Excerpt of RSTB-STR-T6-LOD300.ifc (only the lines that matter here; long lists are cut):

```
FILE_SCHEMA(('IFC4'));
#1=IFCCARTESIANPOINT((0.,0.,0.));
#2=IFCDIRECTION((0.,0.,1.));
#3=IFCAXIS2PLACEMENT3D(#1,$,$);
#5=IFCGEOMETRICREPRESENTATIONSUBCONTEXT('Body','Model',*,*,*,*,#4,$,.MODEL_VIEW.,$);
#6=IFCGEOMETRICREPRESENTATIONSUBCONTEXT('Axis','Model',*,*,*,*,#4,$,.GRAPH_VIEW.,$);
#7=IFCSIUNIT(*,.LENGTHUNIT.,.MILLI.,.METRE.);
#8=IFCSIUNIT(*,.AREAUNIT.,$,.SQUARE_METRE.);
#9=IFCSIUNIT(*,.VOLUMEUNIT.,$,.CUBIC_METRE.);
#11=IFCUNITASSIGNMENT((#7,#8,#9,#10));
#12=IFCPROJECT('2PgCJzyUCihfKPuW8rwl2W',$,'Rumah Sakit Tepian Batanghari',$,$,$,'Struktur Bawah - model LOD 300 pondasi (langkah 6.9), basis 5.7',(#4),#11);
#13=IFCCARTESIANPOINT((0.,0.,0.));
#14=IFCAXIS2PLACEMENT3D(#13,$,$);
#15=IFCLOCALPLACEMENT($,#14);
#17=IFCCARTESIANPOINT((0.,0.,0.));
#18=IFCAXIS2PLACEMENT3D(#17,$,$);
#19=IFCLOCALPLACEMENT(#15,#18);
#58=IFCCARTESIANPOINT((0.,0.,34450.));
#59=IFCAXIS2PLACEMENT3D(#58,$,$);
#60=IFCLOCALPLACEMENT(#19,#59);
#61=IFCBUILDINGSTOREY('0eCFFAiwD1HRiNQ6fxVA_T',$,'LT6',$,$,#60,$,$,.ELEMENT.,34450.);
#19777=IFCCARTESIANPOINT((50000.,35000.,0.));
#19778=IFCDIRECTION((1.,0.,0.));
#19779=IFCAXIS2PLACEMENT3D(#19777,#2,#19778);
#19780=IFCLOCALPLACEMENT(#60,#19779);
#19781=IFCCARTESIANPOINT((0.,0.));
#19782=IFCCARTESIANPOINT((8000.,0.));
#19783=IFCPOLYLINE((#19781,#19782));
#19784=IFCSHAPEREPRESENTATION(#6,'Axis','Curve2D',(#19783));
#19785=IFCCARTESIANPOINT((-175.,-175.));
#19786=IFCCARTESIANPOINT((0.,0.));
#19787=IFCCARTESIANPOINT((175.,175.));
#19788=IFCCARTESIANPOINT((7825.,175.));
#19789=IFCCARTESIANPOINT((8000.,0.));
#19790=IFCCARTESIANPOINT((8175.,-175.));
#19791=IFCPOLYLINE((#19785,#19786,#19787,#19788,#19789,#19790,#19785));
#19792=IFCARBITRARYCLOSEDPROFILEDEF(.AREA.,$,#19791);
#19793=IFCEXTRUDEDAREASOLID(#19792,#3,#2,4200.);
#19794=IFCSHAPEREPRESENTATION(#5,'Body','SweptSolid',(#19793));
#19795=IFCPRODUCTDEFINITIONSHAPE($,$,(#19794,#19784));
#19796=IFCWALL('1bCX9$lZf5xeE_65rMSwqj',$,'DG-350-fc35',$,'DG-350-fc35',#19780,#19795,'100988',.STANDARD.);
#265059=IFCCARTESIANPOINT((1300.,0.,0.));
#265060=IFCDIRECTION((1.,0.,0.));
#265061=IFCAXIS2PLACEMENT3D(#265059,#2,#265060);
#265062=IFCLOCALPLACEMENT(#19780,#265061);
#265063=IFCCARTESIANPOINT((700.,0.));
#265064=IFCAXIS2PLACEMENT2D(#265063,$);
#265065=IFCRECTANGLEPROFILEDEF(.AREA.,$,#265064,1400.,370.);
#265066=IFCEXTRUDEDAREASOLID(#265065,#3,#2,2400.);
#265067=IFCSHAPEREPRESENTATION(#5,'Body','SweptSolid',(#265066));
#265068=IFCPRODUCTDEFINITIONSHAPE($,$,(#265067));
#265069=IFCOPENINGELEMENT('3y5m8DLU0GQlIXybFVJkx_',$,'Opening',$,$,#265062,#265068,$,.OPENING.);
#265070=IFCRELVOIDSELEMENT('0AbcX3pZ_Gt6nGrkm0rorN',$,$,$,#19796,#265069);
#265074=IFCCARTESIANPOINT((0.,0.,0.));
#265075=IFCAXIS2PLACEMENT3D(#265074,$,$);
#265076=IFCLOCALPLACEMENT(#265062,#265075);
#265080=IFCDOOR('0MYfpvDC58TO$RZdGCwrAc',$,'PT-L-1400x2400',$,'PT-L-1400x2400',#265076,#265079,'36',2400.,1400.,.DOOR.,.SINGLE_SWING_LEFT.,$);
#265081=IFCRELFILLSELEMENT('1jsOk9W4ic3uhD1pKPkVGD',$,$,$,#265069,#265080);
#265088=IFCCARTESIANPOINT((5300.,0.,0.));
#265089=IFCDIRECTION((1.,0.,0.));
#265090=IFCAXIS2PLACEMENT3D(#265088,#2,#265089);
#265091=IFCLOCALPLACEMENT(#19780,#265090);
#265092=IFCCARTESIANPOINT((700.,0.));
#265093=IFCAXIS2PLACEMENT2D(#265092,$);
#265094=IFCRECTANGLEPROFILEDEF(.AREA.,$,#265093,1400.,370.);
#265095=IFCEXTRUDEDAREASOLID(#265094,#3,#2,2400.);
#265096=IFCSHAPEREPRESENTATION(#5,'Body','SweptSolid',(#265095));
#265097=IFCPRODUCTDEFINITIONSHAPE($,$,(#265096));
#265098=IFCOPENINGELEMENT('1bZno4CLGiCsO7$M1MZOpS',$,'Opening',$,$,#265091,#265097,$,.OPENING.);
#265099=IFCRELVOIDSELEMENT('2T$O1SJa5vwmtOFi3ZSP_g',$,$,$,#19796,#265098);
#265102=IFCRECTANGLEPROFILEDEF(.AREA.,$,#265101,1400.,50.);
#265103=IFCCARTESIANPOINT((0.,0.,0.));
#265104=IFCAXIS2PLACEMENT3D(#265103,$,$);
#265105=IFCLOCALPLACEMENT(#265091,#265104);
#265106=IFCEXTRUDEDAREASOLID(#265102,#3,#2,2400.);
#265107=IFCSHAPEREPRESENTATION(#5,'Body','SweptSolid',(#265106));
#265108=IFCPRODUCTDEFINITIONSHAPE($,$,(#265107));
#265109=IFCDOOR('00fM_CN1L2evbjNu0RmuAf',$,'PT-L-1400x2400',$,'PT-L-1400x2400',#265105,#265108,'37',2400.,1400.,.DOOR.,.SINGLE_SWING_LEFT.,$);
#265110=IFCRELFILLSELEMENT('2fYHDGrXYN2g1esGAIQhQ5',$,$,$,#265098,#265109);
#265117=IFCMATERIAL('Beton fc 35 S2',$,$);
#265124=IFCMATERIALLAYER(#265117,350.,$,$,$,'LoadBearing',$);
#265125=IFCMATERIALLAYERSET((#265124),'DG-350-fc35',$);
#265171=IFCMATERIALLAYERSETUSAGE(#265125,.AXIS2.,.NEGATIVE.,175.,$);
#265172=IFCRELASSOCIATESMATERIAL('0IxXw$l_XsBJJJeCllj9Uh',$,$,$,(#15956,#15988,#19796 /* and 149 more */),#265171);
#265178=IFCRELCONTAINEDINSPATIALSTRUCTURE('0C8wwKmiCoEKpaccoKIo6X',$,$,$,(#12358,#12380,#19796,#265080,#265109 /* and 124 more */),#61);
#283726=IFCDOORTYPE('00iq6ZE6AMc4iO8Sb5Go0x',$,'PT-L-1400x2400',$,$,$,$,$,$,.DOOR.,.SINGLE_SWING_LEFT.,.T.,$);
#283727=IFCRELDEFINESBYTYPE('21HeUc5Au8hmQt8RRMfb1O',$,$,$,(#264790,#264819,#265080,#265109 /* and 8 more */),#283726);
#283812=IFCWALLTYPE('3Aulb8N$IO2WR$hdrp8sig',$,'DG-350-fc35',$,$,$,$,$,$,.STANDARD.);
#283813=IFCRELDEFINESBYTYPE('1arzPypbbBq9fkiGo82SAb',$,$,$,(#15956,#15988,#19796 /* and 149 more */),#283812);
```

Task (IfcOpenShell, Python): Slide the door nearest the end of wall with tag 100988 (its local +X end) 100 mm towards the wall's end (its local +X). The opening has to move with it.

```python
import ifcopenshell
import ifcopenshell.api.geometry
import ifcopenshell.util.placement
import ifcopenshell.util.unit

model = ifcopenshell.open("RSTB-STR-T6-LOD300.ifc")
unit_scale = ifcopenshell.util.unit.calculate_unit_scale(model)

door = model.by_guid("00fM_CN1L2evbjNu0RmuAf")
opening = door.FillsVoids[0].RelatingOpeningElement
wall = opening.VoidsElements[0].RelatingBuildingElement

wall_matrix = ifcopenshell.util.placement.get_local_placement(wall.ObjectPlacement)
shift = wall_matrix[:3, 0] * 0.1 / unit_scale
before = ifcopenshell.util.placement.get_local_placement(door.ObjectPlacement)[:3, 3].copy()

# The door is placed relative to its opening, so it follows when the opening moves.
matrix = ifcopenshell.util.placement.get_local_placement(opening.ObjectPlacement)
matrix[:3, 3] += shift
ifcopenshell.api.geometry.edit_object_placement(
    model, product=opening, matrix=matrix, is_si=False, should_transform_children=True
)

after = ifcopenshell.util.placement.get_local_placement(door.ObjectPlacement)[:3, 3]
print("door moved by", (after - before).round(3) + 0.0)

model.write("RSTB-STR-T6-LOD300_rev.ifc")
```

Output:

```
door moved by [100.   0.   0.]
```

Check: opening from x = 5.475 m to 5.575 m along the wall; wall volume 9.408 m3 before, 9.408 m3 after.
